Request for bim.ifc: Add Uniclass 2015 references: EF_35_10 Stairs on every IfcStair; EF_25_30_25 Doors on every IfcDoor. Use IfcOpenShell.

First a look at what the model holds.

```python
import ifcopenshell

model = ifcopenshell.open("bim.ifc")
print(model.schema)
print("classifications:", [c.Name for c in model.by_type("IfcClassification")])
for ifc_class in ("IfcDoor", "IfcRoof", "IfcStair", "IfcWall", "IfcWindow"):
    print(ifc_class, len(model.by_type(ifc_class)))
```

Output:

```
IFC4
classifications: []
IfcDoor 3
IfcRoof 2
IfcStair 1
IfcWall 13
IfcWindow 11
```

```python
import ifcopenshell
import ifcopenshell.api.classification

model = ifcopenshell.open("bim.ifc")

system = ifcopenshell.api.classification.add_classification(model, classification="Uniclass 2015")

codes = {
    "IfcStair": ("EF_35_10", "Stairs"),
    "IfcDoor": ("EF_25_30_25", "Doors"),
}
for ifc_class, (code, name) in codes.items():
    products = model.by_type(ifc_class)
    ifcopenshell.api.classification.add_reference(
        model, products=products, classification=system, identification=code, name=name
    )
    print(code, len(products))

model.write("bim_rev.ifc")
```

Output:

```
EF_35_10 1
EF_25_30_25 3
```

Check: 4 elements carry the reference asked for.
